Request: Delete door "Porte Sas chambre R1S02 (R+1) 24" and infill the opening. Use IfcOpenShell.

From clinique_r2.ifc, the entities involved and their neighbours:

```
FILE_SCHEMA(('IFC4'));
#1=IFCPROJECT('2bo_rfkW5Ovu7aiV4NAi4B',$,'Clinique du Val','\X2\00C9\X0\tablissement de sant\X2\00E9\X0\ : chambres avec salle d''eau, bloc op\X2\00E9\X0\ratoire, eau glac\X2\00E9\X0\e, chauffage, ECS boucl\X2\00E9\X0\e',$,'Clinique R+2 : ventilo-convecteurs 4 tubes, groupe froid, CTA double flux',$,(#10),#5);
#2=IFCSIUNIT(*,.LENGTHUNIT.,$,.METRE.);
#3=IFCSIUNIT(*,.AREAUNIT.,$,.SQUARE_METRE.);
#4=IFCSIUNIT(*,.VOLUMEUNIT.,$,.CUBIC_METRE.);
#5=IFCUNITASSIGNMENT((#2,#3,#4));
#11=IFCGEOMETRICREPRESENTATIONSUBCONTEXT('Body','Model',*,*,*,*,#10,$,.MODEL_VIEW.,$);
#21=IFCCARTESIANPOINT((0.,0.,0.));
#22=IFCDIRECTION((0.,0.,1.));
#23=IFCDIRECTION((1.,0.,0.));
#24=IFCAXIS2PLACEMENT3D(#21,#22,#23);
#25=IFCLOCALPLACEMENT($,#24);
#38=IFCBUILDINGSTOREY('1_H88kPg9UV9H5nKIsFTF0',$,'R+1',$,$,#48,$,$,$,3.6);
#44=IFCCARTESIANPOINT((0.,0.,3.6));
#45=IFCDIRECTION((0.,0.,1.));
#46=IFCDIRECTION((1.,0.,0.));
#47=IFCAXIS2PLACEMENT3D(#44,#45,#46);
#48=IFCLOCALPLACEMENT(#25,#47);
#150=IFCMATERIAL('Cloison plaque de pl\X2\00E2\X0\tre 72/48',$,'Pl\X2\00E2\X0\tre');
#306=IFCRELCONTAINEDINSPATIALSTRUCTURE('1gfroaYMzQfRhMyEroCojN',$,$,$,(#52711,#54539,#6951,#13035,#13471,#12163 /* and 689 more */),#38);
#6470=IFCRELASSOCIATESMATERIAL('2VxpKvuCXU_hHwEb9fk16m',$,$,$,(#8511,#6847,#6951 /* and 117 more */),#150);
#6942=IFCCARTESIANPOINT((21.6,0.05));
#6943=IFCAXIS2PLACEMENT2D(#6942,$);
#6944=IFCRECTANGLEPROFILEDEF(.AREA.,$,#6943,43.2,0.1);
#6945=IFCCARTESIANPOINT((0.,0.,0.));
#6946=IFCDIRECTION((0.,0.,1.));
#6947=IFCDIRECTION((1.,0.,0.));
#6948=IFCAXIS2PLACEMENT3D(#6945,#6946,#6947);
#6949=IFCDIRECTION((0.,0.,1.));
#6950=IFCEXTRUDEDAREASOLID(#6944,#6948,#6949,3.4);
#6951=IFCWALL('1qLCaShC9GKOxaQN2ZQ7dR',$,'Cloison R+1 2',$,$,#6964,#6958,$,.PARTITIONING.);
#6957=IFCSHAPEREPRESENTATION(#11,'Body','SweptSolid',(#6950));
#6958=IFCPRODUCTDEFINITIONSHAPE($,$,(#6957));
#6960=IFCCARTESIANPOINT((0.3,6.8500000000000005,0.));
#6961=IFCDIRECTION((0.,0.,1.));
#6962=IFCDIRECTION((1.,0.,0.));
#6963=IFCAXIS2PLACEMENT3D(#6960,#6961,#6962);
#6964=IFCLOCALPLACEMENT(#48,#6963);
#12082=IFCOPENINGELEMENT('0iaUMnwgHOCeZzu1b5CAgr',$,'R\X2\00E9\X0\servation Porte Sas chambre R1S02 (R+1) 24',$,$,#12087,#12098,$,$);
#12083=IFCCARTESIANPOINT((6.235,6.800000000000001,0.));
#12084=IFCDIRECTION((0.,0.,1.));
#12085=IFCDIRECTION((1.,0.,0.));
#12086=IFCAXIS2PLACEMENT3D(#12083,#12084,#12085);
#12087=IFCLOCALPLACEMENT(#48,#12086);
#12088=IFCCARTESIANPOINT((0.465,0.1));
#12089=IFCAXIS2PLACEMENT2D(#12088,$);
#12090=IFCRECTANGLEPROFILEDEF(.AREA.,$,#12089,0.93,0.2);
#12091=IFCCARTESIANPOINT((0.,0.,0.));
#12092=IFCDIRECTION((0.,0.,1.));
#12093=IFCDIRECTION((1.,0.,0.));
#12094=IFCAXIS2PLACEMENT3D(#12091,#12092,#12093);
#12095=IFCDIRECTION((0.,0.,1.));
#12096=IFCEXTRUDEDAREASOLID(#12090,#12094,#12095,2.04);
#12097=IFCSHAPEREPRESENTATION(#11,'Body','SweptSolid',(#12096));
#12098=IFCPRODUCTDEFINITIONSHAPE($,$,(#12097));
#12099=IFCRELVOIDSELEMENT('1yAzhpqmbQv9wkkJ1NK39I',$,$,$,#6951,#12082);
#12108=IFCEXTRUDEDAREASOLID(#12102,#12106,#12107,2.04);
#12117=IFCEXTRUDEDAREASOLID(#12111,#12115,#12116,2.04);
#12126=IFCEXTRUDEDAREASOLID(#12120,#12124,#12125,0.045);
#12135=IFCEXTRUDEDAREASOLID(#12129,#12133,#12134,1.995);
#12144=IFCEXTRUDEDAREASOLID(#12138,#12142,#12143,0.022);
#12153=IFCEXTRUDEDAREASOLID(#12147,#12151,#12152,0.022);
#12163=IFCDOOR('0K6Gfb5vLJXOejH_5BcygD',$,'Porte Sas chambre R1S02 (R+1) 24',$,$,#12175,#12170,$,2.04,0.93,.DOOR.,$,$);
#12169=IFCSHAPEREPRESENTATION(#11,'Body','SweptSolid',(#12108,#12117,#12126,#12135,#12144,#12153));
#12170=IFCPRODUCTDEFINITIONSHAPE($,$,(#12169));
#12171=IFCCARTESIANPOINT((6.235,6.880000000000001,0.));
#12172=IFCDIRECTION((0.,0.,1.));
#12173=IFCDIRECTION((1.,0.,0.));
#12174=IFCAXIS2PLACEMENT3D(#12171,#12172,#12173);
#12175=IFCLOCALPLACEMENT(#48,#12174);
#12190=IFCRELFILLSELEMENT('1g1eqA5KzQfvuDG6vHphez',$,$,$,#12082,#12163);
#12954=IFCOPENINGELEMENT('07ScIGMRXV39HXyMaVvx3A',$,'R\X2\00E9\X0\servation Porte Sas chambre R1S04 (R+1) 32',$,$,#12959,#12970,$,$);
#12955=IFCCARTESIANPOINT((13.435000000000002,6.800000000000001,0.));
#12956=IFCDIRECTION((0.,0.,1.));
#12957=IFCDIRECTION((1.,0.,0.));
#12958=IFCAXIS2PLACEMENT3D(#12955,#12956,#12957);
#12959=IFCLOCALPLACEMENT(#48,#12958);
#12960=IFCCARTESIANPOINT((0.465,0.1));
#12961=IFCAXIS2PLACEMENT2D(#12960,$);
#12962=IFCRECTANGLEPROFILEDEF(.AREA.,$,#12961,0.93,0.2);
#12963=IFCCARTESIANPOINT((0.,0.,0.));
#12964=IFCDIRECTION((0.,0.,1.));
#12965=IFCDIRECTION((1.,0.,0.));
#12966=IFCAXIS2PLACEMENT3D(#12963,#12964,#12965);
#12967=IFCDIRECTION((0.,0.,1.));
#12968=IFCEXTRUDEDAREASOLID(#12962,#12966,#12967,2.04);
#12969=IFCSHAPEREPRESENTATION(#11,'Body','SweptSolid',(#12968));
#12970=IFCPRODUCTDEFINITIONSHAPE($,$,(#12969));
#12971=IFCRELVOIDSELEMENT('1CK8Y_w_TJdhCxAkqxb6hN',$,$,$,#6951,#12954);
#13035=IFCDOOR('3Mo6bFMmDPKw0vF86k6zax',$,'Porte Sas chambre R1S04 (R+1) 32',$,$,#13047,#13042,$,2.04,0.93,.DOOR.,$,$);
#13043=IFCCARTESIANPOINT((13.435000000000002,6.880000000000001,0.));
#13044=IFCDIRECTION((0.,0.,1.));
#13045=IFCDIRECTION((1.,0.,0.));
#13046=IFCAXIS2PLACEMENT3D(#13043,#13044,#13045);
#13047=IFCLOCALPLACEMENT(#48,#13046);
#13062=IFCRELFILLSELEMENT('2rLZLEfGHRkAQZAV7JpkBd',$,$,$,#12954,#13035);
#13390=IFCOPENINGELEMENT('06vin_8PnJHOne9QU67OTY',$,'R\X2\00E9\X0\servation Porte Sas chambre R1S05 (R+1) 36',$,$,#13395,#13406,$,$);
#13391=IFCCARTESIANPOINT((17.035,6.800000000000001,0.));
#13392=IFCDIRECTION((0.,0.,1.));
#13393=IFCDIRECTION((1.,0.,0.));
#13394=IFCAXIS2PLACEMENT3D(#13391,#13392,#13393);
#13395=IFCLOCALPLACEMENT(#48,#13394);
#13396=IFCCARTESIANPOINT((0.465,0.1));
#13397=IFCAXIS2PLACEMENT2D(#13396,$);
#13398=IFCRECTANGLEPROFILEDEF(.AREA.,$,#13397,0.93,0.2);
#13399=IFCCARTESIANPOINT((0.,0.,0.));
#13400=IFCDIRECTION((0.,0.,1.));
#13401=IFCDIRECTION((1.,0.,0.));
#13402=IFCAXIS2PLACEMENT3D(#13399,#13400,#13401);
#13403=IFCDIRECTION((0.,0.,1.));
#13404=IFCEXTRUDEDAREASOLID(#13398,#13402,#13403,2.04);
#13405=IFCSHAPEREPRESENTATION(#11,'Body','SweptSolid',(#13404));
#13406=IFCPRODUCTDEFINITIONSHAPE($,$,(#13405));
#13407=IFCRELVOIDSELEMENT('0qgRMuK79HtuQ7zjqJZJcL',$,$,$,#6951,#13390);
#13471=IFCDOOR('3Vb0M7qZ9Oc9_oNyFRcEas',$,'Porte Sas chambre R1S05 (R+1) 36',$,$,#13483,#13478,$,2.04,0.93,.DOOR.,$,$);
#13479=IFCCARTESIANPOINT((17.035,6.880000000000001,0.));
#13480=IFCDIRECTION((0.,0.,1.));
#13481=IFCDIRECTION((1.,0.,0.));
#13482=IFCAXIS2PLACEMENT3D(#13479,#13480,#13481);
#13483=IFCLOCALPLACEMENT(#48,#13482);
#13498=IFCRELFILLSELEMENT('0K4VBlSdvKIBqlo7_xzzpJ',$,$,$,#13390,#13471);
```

```python
import ifcopenshell
import ifcopenshell.api.feature
import ifcopenshell.api.root
import ifcopenshell.geom
import ifcopenshell.util.shape

model = ifcopenshell.open("clinique_r2.ifc")
settings = ifcopenshell.geom.settings()


def volume(element):
    """Net volume in cubic metres, openings subtracted."""
    shape = ifcopenshell.geom.create_shape(settings, element)
    return ifcopenshell.util.shape.get_volume(shape.geometry)


door = model.by_guid("0K6Gfb5vLJXOejH_5BcygD")
opening = door.FillsVoids[0].RelatingOpeningElement
wall = opening.VoidsElements[0].RelatingBuildingElement
before = volume(wall)

ifcopenshell.api.root.remove_product(model, product=door)
ifcopenshell.api.feature.remove_feature(model, feature=opening)

after = volume(wall)

print(f"wall volume {before:.3f} -> {after:.3f} m3")

model.write("clinique_r2_updated.ifc")
```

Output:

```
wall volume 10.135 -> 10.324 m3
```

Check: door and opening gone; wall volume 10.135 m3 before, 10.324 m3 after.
